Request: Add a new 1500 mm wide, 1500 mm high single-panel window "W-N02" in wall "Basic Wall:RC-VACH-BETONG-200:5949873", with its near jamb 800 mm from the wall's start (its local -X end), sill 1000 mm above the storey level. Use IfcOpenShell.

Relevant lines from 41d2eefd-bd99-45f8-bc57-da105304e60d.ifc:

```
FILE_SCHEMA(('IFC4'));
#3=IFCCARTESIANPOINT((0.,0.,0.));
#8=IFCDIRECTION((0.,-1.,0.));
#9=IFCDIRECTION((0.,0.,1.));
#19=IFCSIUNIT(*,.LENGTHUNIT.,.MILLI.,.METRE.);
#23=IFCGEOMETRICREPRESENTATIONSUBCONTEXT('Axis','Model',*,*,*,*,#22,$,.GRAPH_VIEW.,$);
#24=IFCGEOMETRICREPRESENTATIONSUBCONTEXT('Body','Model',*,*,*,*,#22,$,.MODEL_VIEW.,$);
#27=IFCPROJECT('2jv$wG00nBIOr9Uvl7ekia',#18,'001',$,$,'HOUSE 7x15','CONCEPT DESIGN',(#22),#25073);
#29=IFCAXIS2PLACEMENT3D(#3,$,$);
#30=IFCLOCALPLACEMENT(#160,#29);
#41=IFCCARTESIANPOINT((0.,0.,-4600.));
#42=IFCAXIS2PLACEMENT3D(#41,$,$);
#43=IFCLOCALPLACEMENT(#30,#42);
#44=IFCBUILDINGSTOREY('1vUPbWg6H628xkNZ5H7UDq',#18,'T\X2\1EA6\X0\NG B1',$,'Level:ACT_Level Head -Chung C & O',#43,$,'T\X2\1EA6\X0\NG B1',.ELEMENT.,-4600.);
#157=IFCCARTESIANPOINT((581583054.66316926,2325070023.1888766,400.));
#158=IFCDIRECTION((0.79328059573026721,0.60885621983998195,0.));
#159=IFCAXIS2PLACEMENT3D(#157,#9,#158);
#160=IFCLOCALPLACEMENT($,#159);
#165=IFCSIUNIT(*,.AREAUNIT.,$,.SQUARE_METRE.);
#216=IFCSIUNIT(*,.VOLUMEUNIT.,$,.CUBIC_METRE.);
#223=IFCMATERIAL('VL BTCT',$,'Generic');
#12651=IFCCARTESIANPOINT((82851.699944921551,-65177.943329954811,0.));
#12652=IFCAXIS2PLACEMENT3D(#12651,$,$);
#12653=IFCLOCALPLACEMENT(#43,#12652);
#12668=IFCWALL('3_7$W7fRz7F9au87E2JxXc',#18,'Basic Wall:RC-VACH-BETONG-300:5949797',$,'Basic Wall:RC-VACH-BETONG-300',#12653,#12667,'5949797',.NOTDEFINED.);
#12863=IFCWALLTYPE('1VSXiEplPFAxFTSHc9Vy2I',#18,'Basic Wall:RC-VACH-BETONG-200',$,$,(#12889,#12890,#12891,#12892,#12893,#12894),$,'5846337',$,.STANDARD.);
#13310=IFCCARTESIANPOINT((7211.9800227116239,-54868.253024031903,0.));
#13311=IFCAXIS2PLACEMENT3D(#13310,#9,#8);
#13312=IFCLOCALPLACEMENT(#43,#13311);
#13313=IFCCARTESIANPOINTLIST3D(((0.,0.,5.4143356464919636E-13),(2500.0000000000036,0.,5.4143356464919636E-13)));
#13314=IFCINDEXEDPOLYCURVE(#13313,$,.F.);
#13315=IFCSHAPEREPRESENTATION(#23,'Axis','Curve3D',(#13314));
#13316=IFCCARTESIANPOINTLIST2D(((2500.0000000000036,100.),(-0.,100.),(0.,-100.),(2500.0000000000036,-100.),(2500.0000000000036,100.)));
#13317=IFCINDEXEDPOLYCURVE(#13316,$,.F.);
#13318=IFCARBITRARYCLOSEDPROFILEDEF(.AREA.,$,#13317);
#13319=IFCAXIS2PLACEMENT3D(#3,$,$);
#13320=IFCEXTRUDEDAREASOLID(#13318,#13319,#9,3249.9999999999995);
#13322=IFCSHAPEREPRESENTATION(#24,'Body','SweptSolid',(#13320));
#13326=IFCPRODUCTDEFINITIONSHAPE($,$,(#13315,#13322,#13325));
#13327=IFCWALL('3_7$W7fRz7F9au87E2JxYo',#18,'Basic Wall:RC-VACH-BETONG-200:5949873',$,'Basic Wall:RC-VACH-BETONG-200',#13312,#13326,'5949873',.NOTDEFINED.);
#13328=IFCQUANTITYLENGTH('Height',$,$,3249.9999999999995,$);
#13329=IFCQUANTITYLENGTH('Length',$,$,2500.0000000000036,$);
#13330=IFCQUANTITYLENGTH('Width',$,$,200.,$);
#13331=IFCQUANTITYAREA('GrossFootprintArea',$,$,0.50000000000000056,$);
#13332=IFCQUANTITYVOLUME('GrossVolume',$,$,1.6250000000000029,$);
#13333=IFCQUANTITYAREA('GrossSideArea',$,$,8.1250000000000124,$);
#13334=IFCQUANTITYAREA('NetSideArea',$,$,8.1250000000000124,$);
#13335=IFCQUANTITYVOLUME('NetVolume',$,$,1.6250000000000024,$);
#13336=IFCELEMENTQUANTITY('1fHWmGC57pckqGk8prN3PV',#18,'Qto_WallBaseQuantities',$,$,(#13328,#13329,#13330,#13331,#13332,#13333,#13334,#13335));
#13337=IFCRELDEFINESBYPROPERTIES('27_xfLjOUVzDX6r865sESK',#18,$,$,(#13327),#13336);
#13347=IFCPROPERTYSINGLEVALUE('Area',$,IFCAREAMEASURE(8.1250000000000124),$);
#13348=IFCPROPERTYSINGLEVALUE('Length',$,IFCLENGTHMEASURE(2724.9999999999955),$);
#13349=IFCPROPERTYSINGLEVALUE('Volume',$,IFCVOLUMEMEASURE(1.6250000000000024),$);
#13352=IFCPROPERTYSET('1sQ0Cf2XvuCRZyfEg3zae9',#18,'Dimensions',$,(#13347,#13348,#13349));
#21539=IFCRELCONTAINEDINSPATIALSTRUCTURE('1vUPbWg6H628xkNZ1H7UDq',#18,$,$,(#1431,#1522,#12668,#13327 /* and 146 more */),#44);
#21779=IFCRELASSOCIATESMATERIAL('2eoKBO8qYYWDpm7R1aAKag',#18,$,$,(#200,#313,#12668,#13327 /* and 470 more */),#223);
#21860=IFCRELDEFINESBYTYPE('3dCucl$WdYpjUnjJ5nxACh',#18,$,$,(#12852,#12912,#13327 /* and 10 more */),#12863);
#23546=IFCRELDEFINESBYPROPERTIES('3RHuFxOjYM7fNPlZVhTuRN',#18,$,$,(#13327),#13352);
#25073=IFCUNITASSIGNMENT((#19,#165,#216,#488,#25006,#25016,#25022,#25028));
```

```python
import numpy as np
import ifcopenshell
import ifcopenshell.api.feature
import ifcopenshell.api.geometry
import ifcopenshell.api.pset
import ifcopenshell.api.root
import ifcopenshell.api.spatial
import ifcopenshell.geom
import ifcopenshell.util.element
import ifcopenshell.util.placement
import ifcopenshell.util.representation
import ifcopenshell.util.shape
import ifcopenshell.util.unit

model = ifcopenshell.open("41d2eefd-bd99-45f8-bc57-da105304e60d.ifc")
unit_scale = ifcopenshell.util.unit.calculate_unit_scale(model)
area_scale = ifcopenshell.util.unit.calculate_unit_scale(model, "AREAUNIT")
volume_scale = ifcopenshell.util.unit.calculate_unit_scale(model, "VOLUMEUNIT")
settings = ifcopenshell.geom.settings()


def volume(element):
    """Net volume in cubic metres, openings subtracted."""
    shape = ifcopenshell.geom.create_shape(settings, element)
    return ifcopenshell.util.shape.get_volume(shape.geometry)


wall = model.by_guid("3_7$W7fRz7F9au87E2JxYo")
storey = ifcopenshell.util.element.get_container(wall, ifc_class="IfcBuildingStorey")
context = ifcopenshell.util.representation.get_context(model, "Model", "Body", "MODEL_VIEW")
before = volume(wall)

width, height, from_end, sill = 1.5, 1.5, 0.8, 1  # metres

# The wall runs along its own X axis, and the end named is its -X end.
wall_shape = ifcopenshell.geom.create_shape(settings, wall)
x, y, z = ifcopenshell.util.shape.get_vertices(wall_shape.geometry).T
start = x.min() + from_end
face, thickness = float(y.min()), float(y.max() - y.min())
wall_matrix = ifcopenshell.util.placement.get_local_placement(wall.ObjectPlacement)
level = ifcopenshell.util.placement.get_local_placement(storey.ObjectPlacement)[2, 3]


def in_wall(x, y):
    """Placement at x, y metres in the wall's axes, at sill height."""
    matrix = wall_matrix.copy()
    matrix[:, 3] = wall_matrix @ np.array([x / unit_scale, y / unit_scale, 0.0, 1.0])
    matrix[2, 3] = level + sill / unit_scale
    return matrix


# Opening: a box that overshoots both wall faces by 50 mm.
opening = ifcopenshell.api.root.create_entity(model, ifc_class="IfcOpeningElement", predefined_type="OPENING")
box = ifcopenshell.api.geometry.add_wall_representation(
    model, context=context, length=width, height=height, thickness=thickness + 0.1
)
ifcopenshell.api.geometry.assign_representation(model, product=opening, representation=box)
ifcopenshell.api.geometry.edit_object_placement(model, product=opening, matrix=in_wall(start, face - 0.05), is_si=False)
ifcopenshell.api.feature.add_feature(model, feature=opening, element=wall)

window = ifcopenshell.api.root.create_entity(model, ifc_class="IfcWindow", name="W-N02", predefined_type="WINDOW")
window.OverallWidth, window.OverallHeight = width / unit_scale, height / unit_scale
window.PartitioningType = "SINGLE_PANEL"
body = ifcopenshell.api.geometry.add_window_representation(
    model,
    context=context,
    overall_width=window.OverallWidth,
    overall_height=window.OverallHeight,
    partition_type="SINGLE_PANEL",
)
ifcopenshell.api.geometry.assign_representation(model, product=window, representation=body)
ifcopenshell.api.spatial.assign_container(model, products=[window], relating_structure=storey)
ifcopenshell.api.feature.add_filling(model, opening=opening, element=window)

# Centre the window in the wall's thickness.
ifcopenshell.api.geometry.edit_object_placement(model, product=window, matrix=in_wall(start, face), is_si=False)
window_shape = ifcopenshell.geom.create_shape(settings, window)
depth = ifcopenshell.util.shape.get_vertices(window_shape.geometry)[:, 1]
offset = face + thickness / 2 - (depth.min() + depth.max()) / 2
ifcopenshell.api.geometry.edit_object_placement(model, product=window, matrix=in_wall(start, offset), is_si=False)

after = volume(wall)

# Update the wall's stored quantities.
qto = model.by_id(ifcopenshell.util.element.get_pset(wall, "Qto_WallBaseQuantities", should_inherit=False)["id"])
ifcopenshell.api.pset.edit_qto(model, qto=qto, properties={
    "NetSideArea": after / thickness / area_scale,
    "NetVolume": after / volume_scale,
})
pset = model.by_id(ifcopenshell.util.element.get_pset(wall, "Dimensions", should_inherit=False)["id"])
ifcopenshell.api.pset.edit_pset(model, pset=pset, properties={
    "Area": model.create_entity("IfcAreaMeasure", after / thickness / area_scale),
    "Volume": model.create_entity("IfcVolumeMeasure", after / volume_scale),
})

print(f"wall volume {before:.3f} -> {after:.3f} m3")

model.write("41d2eefd-bd99-45f8-bc57-da105304e60d_updated.ifc")
```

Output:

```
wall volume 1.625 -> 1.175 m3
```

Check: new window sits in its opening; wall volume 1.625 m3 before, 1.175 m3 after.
